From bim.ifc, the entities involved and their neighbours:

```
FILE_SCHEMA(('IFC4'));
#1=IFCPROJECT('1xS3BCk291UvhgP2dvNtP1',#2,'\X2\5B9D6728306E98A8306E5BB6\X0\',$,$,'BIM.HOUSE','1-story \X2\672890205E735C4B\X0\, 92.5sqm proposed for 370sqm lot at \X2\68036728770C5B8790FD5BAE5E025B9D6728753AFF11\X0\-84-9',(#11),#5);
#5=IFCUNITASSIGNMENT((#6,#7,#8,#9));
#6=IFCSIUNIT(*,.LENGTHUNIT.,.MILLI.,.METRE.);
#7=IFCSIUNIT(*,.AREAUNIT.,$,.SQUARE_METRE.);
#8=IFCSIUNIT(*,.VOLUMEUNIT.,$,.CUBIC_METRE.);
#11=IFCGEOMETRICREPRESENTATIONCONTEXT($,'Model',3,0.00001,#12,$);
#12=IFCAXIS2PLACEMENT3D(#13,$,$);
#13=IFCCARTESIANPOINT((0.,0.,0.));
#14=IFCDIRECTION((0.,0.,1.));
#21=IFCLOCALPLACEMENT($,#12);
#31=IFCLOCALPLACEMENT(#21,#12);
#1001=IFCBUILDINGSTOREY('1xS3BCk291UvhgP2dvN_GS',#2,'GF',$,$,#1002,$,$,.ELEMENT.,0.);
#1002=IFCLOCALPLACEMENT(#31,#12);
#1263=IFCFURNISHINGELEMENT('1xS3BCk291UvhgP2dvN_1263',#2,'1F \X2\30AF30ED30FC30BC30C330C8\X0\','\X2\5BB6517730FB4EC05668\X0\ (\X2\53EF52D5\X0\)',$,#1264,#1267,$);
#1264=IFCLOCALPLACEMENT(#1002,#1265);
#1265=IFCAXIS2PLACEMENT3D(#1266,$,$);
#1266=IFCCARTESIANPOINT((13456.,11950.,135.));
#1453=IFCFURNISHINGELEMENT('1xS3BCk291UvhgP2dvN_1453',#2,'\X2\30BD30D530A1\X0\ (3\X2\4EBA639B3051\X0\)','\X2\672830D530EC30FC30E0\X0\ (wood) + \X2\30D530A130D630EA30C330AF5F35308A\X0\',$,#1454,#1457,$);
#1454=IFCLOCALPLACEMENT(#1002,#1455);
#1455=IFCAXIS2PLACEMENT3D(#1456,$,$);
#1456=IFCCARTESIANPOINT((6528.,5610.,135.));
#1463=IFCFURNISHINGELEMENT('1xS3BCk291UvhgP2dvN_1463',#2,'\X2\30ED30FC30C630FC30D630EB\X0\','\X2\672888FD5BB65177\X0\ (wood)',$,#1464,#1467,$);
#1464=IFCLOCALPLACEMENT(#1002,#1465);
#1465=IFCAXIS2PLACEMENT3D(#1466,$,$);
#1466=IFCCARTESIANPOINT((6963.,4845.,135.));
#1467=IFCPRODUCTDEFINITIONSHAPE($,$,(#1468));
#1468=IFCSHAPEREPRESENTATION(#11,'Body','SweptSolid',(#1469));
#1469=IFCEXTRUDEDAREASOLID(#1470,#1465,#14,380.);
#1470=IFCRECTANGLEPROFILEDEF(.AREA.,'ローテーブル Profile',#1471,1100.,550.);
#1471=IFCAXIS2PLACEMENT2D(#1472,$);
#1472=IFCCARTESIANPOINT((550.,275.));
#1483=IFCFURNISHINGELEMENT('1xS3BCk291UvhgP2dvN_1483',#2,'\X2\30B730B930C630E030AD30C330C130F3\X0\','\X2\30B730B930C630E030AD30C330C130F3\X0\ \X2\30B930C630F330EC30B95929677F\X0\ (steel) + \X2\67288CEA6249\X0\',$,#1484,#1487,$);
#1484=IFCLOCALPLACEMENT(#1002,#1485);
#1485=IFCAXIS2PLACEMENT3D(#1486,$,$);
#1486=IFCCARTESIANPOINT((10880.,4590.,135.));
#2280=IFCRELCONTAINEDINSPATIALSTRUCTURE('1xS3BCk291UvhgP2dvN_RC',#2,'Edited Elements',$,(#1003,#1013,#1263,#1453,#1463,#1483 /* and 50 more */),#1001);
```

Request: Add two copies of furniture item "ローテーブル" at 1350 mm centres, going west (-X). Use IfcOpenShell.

```python
import numpy as np
import ifcopenshell
import ifcopenshell.api.geometry
import ifcopenshell.api.root
import ifcopenshell.util.element
import ifcopenshell.util.placement
import ifcopenshell.util.unit

model = ifcopenshell.open("bim.ifc")
unit_scale = ifcopenshell.util.unit.calculate_unit_scale(model)


def reuse_history(source, copy):
    """copy_class also copies each property set's owner history, people and application; keep the originals."""
    for rel in copy.IsDefinedBy:
        if rel.is_a("IfcRelDefinesByProperties") and (history := rel.RelatingPropertyDefinition.OwnerHistory):
            rel.RelatingPropertyDefinition.OwnerHistory = source.OwnerHistory
            ifcopenshell.util.element.remove_deep2(model, history)


source = model.by_guid("1xS3BCk291UvhgP2dvN_1463")
base = ifcopenshell.util.placement.get_local_placement(source.ObjectPlacement)
step = np.array([-1.0, 0.0, 0.0]) * 1.35 / unit_scale

for i in range(1, 3):
    copy = ifcopenshell.api.root.copy_class(model, product=source)
    copy.Representation = ifcopenshell.util.element.copy_deep(
        model, source.Representation, exclude=["IfcGeometricRepresentationContext", "IfcRepresentationMap"]
    )
    reuse_history(source, copy)
    matrix = base.copy()
    matrix[:3, 3] += i * step
    print("added at", matrix[:3, 3].round(3) + 0.0)
    ifcopenshell.api.geometry.edit_object_placement(model, product=copy, matrix=matrix, is_si=False)

model.write("bim_rev.ifc")
```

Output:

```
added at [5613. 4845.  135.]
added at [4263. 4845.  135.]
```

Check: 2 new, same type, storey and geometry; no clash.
